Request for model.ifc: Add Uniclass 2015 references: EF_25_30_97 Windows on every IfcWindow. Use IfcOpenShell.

First a look at what the model holds.

```python
import ifcopenshell

model = ifcopenshell.open("model.ifc")
print(model.schema)
print("classifications:", [c.Name for c in model.by_type("IfcClassification")])
for ifc_class in ("IfcDoor", "IfcRoof", "IfcStair", "IfcWall", "IfcWindow"):
    print(ifc_class, len(model.by_type(ifc_class)))
```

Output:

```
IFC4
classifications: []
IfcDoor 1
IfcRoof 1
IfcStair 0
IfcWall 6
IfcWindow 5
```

```python
import ifcopenshell
import ifcopenshell.api.classification

model = ifcopenshell.open("model.ifc")

system = ifcopenshell.api.classification.add_classification(model, classification="Uniclass 2015")

codes = {
    "IfcWindow": ("EF_25_30_97", "Windows"),
}
for ifc_class, (code, name) in codes.items():
    products = model.by_type(ifc_class)
    ifcopenshell.api.classification.add_reference(
        model, products=products, classification=system, identification=code, name=name
    )
    print(code, len(products))

model.write("model-out.ifc")
```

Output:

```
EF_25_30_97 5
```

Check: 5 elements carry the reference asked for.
